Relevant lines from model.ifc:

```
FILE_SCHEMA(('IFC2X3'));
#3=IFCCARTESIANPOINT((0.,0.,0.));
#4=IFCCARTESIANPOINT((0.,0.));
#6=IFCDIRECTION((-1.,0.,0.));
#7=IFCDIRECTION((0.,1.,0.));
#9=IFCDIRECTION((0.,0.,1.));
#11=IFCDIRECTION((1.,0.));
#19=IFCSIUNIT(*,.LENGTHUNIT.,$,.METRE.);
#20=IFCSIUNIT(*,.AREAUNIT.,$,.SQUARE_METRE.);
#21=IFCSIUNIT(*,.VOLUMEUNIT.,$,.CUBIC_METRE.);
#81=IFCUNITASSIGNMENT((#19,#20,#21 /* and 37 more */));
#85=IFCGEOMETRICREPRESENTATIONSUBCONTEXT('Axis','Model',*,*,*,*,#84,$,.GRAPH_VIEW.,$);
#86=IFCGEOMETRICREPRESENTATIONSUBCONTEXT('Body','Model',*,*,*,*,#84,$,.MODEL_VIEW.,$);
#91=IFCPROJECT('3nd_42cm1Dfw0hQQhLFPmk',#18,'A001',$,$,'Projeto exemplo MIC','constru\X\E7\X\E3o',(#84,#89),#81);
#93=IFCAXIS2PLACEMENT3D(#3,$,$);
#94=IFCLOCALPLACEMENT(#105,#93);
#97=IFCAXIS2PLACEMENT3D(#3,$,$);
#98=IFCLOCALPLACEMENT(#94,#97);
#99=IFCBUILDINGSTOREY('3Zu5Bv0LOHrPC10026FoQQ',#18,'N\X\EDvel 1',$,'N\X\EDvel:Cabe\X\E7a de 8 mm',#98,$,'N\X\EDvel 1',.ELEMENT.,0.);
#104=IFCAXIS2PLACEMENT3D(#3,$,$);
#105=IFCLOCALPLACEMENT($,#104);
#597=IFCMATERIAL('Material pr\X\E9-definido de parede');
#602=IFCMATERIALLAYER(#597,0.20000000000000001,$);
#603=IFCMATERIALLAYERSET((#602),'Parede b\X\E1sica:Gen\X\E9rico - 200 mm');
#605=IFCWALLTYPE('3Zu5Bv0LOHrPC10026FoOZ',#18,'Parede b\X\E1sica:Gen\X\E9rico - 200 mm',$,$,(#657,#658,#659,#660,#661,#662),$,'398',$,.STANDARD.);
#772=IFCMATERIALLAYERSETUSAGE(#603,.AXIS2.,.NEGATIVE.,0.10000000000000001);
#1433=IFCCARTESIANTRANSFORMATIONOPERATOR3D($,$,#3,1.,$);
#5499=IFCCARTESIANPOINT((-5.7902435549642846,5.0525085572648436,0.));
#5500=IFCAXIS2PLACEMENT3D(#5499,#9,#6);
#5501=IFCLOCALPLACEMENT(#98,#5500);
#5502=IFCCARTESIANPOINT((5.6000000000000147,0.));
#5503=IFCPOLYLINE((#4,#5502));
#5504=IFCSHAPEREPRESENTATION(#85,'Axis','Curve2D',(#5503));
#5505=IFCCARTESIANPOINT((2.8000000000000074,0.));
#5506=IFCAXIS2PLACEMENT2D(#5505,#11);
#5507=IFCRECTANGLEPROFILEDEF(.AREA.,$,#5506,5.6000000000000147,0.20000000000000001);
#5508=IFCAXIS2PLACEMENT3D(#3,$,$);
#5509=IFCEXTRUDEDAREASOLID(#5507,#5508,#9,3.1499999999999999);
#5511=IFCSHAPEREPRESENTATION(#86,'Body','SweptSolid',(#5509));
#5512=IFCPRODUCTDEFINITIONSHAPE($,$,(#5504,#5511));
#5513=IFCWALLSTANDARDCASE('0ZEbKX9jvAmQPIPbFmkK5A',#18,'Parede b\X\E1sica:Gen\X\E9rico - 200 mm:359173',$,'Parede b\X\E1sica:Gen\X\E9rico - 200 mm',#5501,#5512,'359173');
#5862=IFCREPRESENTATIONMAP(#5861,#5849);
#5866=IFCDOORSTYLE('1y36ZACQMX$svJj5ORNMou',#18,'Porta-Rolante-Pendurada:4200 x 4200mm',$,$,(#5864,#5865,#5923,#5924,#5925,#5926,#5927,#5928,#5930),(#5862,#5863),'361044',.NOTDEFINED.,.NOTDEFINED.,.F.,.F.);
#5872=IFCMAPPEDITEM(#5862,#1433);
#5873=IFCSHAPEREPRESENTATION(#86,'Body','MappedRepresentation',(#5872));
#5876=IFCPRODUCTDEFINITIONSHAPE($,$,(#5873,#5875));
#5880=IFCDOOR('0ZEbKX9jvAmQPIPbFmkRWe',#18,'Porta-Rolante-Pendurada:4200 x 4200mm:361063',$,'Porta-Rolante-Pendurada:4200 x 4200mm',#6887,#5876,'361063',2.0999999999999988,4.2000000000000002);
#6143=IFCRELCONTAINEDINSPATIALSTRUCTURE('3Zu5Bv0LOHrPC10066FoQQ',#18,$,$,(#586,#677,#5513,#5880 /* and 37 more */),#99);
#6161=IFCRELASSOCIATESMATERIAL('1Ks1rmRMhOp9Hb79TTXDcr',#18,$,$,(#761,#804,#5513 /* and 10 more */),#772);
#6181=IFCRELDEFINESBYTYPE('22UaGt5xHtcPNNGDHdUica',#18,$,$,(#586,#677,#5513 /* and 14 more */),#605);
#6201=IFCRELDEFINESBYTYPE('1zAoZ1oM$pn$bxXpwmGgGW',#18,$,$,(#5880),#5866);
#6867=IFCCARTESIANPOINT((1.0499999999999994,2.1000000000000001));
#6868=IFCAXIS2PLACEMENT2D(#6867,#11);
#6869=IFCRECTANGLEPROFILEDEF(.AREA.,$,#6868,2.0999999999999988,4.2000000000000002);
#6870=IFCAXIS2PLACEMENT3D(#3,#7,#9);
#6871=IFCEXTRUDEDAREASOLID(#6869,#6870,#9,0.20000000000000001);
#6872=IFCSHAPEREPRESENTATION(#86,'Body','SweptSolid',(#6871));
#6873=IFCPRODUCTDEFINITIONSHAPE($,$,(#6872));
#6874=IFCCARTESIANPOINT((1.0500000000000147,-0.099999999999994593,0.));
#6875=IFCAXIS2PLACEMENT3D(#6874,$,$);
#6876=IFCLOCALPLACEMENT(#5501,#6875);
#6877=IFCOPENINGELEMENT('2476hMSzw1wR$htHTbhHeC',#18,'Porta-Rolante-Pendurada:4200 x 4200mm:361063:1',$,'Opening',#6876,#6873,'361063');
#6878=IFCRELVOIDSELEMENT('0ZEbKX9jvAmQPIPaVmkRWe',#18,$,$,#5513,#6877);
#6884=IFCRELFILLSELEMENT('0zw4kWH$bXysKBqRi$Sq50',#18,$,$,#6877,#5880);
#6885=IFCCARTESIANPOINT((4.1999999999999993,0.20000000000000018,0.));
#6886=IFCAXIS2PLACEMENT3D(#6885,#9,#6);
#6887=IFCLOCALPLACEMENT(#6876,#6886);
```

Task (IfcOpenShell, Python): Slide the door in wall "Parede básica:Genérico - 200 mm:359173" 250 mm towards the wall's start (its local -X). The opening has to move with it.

```python
import ifcopenshell
import ifcopenshell.api.geometry
import ifcopenshell.util.placement
import ifcopenshell.util.unit

model = ifcopenshell.open("model.ifc")
unit_scale = ifcopenshell.util.unit.calculate_unit_scale(model)

door = model.by_guid("0ZEbKX9jvAmQPIPbFmkRWe")
opening = door.FillsVoids[0].RelatingOpeningElement
wall = opening.VoidsElements[0].RelatingBuildingElement

wall_matrix = ifcopenshell.util.placement.get_local_placement(wall.ObjectPlacement)
shift = wall_matrix[:3, 0] * -0.25 / unit_scale
before = ifcopenshell.util.placement.get_local_placement(door.ObjectPlacement)[:3, 3].copy()

# The door is placed relative to its opening, so it follows when the opening moves.
matrix = ifcopenshell.util.placement.get_local_placement(opening.ObjectPlacement)
matrix[:3, 3] += shift
ifcopenshell.api.geometry.edit_object_placement(
    model, product=opening, matrix=matrix, is_si=False, should_transform_children=True
)

after = ifcopenshell.util.placement.get_local_placement(door.ObjectPlacement)[:3, 3]
print("door moved by", (after - before).round(3) + 0.0)

model.write("model_v2.ifc")
```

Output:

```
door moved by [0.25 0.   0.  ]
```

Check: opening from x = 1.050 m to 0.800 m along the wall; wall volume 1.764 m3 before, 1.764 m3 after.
